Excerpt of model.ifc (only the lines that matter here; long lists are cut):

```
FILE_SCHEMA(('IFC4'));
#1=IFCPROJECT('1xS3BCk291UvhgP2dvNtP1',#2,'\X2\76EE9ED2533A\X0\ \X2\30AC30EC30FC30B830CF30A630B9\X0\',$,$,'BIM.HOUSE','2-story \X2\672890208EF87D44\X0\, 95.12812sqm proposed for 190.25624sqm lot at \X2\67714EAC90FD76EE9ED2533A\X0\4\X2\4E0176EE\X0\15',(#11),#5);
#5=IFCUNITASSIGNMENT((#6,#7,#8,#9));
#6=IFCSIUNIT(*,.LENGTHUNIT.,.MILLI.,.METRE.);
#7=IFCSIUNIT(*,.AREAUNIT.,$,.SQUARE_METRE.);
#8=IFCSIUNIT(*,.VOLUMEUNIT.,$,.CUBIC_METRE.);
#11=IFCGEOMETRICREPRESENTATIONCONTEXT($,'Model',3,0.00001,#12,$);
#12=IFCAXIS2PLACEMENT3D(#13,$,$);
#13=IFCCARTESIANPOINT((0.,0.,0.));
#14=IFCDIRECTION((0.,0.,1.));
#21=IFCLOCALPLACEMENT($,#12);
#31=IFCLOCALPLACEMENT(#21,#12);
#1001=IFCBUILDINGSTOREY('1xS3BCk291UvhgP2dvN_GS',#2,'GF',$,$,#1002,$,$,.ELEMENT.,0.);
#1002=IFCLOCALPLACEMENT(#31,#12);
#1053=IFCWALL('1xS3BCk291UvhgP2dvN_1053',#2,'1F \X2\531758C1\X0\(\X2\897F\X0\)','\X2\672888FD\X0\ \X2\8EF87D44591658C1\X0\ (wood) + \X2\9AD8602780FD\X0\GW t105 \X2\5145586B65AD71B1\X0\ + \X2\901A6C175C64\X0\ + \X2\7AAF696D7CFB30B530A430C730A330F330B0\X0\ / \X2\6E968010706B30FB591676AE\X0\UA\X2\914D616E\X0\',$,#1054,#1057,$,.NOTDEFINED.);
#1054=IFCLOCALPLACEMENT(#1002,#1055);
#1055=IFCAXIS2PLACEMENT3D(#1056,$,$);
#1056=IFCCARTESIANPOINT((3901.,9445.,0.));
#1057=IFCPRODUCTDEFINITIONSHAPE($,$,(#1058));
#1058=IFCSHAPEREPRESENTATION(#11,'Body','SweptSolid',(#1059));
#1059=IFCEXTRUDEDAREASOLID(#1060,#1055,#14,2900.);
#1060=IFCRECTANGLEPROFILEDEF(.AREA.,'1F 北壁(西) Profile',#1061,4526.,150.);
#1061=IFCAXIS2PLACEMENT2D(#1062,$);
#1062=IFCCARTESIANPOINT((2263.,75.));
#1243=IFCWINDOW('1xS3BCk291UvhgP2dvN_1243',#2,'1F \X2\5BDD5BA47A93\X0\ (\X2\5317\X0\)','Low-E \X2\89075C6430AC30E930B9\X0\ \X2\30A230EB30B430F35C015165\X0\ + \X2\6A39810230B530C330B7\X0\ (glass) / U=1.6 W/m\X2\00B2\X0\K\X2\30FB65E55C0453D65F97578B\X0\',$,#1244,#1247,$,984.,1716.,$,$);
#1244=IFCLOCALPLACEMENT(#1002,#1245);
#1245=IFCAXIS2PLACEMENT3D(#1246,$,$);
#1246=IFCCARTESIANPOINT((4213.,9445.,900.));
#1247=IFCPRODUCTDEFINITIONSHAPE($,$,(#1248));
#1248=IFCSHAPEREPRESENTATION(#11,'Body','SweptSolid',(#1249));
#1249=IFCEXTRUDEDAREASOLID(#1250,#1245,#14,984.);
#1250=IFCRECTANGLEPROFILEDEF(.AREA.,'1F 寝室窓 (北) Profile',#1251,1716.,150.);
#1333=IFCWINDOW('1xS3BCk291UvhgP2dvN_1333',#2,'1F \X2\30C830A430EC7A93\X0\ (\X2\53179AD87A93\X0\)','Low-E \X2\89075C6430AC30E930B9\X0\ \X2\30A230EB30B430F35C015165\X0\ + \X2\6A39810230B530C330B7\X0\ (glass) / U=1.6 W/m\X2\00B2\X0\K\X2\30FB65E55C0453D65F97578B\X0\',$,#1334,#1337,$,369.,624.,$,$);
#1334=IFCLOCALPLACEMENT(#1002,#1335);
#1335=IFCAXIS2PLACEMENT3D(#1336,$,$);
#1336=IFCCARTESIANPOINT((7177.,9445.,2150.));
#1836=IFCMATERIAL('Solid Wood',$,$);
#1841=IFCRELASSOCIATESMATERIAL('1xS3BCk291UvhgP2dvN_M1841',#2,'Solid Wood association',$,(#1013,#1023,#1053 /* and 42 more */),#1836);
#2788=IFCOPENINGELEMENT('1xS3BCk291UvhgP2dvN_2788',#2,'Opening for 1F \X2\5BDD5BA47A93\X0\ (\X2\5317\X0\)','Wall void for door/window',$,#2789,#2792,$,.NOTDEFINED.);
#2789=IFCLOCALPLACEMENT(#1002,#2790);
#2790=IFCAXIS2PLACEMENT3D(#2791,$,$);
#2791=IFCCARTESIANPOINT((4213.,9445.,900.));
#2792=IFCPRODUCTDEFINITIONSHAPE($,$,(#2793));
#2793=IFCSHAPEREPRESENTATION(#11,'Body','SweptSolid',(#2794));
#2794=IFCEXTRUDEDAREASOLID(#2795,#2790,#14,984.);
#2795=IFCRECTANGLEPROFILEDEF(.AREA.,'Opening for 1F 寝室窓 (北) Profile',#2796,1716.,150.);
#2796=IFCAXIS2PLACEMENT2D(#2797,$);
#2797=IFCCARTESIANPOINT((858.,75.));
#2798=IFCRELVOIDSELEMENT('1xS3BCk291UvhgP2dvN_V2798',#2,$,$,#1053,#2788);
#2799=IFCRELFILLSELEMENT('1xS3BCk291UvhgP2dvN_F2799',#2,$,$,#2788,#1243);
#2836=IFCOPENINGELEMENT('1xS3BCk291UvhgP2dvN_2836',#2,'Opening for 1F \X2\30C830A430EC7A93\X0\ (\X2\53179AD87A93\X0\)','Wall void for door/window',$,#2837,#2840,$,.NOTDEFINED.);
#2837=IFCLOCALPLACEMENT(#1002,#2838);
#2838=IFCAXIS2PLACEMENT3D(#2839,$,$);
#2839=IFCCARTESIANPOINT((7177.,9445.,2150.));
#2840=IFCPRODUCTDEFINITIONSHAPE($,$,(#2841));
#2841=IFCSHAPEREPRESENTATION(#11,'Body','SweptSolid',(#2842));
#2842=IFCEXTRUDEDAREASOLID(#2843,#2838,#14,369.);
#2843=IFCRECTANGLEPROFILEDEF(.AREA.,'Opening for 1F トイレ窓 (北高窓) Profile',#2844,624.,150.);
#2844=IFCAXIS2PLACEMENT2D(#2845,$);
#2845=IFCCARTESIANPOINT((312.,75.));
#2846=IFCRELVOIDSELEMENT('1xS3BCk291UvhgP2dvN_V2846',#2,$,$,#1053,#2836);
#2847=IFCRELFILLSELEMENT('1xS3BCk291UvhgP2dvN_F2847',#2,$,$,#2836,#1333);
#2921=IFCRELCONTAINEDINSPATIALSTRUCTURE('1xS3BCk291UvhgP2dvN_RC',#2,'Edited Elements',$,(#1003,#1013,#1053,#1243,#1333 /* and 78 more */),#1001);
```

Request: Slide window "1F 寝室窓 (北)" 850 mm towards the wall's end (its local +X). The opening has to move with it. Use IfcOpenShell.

```python
import ifcopenshell
import ifcopenshell.api.geometry
import ifcopenshell.util.placement
import ifcopenshell.util.unit

model = ifcopenshell.open("model.ifc")
unit_scale = ifcopenshell.util.unit.calculate_unit_scale(model)

window = model.by_id(1243)
opening = window.FillsVoids[0].RelatingOpeningElement
wall = opening.VoidsElements[0].RelatingBuildingElement

wall_matrix = ifcopenshell.util.placement.get_local_placement(wall.ObjectPlacement)
shift = wall_matrix[:3, 0] * 0.85 / unit_scale
before = ifcopenshell.util.placement.get_local_placement(window.ObjectPlacement)[:3, 3].copy()

# The window is not placed relative to its opening, so move both.
for product in (opening, window):
    matrix = ifcopenshell.util.placement.get_local_placement(product.ObjectPlacement)
    matrix[:3, 3] += shift
    ifcopenshell.api.geometry.edit_object_placement(model, product=product, matrix=matrix, is_si=False)

after = ifcopenshell.util.placement.get_local_placement(window.ObjectPlacement)[:3, 3]
print("window moved by", (after - before).round(3) + 0.0)

model.write("model_rev.ifc")
```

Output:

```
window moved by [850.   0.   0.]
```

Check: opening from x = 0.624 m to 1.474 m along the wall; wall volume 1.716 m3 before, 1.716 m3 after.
